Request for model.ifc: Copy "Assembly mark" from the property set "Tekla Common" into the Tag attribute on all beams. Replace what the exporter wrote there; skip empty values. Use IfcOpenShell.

First a look at what the model holds.

```python
import ifcopenshell
import ifcopenshell.util.element

model = ifcopenshell.open("model.ifc")
print(model.schema)
beams = model.by_type("IfcBeam")
print(len(beams), "beams")
for e in beams[:8]:
    source = ifcopenshell.util.element.get_pset(e, "Tekla Common", "Assembly mark")
    target = e.Tag
    print(e.id(), repr(source), repr(target), sep=" | ")
```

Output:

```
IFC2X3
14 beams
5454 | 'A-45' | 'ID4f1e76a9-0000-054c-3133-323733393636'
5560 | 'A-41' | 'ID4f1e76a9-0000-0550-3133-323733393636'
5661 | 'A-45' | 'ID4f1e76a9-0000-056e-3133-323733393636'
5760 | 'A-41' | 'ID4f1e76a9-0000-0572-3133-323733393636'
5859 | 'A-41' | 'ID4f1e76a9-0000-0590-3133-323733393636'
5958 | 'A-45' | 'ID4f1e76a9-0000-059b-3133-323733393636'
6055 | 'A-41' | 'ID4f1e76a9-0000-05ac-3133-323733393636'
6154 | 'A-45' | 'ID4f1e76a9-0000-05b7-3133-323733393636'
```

```python
import ifcopenshell
import ifcopenshell.util.element

model = ifcopenshell.open("model.ifc")

count = 0
for e in model.by_type("IfcBeam"):
    value = ifcopenshell.util.element.get_pset(e, "Tekla Common", "Assembly mark")
    current = e.Tag
    if not value or not value.strip() or current == value:
        continue
    e.Tag = value
    count += 1

print(count, "beams updated")

model.write("model_v2.ifc")
```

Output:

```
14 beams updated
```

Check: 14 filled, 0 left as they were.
